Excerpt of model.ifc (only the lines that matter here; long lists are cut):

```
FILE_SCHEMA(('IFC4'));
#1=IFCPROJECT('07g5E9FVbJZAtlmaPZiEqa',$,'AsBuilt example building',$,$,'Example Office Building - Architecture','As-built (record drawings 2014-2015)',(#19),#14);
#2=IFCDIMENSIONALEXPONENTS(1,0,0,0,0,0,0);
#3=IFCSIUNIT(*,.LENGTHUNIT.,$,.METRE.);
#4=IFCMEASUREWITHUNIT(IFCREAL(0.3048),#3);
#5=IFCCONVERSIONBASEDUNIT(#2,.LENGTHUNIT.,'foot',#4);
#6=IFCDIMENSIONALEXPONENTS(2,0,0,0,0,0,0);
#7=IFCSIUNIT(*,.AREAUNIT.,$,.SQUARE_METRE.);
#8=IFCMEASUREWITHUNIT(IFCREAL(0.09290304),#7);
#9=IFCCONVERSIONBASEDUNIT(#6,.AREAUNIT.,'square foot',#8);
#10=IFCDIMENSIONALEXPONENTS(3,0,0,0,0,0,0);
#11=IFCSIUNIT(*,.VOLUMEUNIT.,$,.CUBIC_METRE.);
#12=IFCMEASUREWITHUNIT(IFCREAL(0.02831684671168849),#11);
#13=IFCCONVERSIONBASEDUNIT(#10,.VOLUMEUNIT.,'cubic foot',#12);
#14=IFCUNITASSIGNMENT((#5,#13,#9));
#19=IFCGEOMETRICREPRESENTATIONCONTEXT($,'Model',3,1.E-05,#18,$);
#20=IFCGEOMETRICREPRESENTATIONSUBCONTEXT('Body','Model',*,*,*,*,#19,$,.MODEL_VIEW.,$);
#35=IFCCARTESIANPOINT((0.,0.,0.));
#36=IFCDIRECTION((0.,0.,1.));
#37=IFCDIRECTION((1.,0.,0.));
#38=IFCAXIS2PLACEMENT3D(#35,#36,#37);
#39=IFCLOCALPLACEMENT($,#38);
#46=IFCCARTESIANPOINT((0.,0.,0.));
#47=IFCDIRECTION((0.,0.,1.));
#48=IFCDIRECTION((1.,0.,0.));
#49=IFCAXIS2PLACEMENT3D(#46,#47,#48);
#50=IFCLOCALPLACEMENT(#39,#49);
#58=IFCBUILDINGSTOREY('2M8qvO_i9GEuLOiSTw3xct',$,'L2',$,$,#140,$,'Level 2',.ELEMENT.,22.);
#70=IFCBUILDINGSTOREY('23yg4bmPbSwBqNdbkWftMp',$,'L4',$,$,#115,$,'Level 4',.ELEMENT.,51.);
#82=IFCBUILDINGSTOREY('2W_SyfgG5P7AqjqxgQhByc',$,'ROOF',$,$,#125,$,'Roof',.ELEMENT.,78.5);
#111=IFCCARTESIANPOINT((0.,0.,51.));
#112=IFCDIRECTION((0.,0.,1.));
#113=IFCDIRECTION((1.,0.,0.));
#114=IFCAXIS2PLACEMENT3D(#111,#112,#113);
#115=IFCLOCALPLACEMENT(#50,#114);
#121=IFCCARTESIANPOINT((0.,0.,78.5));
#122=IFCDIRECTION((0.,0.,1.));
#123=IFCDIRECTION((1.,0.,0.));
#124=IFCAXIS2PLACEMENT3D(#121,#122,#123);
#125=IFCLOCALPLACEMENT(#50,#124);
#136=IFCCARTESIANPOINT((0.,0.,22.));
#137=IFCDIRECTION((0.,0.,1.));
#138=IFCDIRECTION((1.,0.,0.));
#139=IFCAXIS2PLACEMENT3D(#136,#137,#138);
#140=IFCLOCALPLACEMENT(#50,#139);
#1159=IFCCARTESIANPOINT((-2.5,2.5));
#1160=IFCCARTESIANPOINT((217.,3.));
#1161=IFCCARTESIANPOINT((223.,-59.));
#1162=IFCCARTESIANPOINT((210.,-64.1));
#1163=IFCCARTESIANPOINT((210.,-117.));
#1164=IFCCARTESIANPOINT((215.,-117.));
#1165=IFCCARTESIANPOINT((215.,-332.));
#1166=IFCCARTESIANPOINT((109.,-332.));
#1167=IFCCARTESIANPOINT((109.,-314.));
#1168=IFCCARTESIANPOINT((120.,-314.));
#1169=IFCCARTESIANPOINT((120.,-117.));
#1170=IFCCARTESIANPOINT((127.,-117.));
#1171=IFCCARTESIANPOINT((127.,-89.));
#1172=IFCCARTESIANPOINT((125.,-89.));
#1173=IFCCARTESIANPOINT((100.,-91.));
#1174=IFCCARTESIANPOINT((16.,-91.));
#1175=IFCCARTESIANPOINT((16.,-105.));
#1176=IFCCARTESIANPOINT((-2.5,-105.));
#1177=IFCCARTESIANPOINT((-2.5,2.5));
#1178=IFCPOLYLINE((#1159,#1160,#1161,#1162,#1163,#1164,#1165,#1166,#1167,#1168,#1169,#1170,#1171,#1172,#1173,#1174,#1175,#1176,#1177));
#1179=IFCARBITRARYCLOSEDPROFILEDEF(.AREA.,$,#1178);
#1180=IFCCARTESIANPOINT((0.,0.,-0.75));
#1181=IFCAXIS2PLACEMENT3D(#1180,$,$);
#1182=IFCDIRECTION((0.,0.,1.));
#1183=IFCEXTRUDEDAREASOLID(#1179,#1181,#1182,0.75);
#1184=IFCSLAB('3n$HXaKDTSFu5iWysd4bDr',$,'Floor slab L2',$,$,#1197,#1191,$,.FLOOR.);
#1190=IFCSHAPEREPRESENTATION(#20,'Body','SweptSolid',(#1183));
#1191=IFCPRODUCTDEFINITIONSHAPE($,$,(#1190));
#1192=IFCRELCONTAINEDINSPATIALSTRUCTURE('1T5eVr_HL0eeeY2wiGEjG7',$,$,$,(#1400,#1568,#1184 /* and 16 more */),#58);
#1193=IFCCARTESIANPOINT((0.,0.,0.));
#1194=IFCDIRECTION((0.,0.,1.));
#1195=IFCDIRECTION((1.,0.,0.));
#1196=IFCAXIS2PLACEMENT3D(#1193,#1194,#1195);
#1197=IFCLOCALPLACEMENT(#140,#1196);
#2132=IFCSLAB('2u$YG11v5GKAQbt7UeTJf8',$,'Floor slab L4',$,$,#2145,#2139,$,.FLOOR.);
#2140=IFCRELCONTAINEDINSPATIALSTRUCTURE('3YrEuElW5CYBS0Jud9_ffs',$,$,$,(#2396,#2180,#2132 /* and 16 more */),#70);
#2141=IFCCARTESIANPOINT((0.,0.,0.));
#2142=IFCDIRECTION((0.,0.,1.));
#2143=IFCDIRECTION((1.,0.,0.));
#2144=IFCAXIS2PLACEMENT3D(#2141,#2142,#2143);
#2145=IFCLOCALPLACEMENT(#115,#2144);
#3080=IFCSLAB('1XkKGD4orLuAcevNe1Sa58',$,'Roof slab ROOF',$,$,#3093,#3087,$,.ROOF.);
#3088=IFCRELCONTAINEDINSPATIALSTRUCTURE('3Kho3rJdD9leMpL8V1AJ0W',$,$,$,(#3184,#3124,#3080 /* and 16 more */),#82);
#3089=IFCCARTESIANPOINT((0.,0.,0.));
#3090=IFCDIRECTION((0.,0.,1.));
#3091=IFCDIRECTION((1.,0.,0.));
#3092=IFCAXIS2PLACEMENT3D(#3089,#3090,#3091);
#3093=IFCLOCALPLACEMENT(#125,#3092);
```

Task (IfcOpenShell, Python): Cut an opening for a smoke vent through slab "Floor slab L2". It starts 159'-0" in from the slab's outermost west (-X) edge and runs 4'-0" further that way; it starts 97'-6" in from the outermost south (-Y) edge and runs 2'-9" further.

```python
import numpy as np
import ifcopenshell
import ifcopenshell.api.feature
import ifcopenshell.api.geometry
import ifcopenshell.api.root
import ifcopenshell.geom
import ifcopenshell.util.placement
import ifcopenshell.util.representation
import ifcopenshell.util.shape
import ifcopenshell.util.unit

model = ifcopenshell.open("model.ifc")
unit_scale = ifcopenshell.util.unit.calculate_unit_scale(model)
settings = ifcopenshell.geom.settings()


def volume(element):
    """Net volume in cubic metres, openings subtracted."""
    shape = ifcopenshell.geom.create_shape(settings, element)
    return ifcopenshell.util.shape.get_volume(shape.geometry)


slab = model.by_guid("3n$HXaKDTSFu5iWysd4bDr")
before = volume(slab)

# Extent in the slab's own axes, in metres. The edges named are its -X and -Y sides.
slab_shape = ifcopenshell.geom.create_shape(settings, slab)
vertices = ifcopenshell.util.shape.get_vertices(slab_shape.geometry)
x_min, y_min, bottom = vertices.min(axis=0)
top = vertices[:, 2].max()

opening = ifcopenshell.api.root.create_entity(model, ifc_class="IfcOpeningElement", name="Smoke vent opening", predefined_type="OPENING")
context = ifcopenshell.util.representation.get_context(model, "Model", "Body", "MODEL_VIEW")
width, depth = 1.2192, 0.8382
outline = [(0.0, 0.0), (width, 0.0), (width, depth), (0.0, depth), (0.0, 0.0)]
# Overshoot both faces by 50 mm so the cut is clean.
shape = ifcopenshell.api.geometry.add_slab_representation(
    model, context=context, depth=top - bottom + 0.1, polyline=outline
)
ifcopenshell.api.geometry.assign_representation(model, product=opening, representation=shape)

matrix = ifcopenshell.util.placement.get_local_placement(slab.ObjectPlacement)
matrix[:, 3] = matrix @ np.append(np.array([x_min + 48.4632, y_min + 29.718, bottom - 0.05]) / unit_scale, 1.0)
ifcopenshell.api.geometry.edit_object_placement(model, product=opening, matrix=matrix, is_si=False)
ifcopenshell.api.feature.add_feature(model, feature=opening, element=slab)

after = volume(slab)

print(f"slab volume {before:.3f} -> {after:.3f} m3")

model.write("model_edited.ifc")
```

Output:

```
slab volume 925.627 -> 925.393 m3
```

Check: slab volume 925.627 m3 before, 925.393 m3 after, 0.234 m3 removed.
